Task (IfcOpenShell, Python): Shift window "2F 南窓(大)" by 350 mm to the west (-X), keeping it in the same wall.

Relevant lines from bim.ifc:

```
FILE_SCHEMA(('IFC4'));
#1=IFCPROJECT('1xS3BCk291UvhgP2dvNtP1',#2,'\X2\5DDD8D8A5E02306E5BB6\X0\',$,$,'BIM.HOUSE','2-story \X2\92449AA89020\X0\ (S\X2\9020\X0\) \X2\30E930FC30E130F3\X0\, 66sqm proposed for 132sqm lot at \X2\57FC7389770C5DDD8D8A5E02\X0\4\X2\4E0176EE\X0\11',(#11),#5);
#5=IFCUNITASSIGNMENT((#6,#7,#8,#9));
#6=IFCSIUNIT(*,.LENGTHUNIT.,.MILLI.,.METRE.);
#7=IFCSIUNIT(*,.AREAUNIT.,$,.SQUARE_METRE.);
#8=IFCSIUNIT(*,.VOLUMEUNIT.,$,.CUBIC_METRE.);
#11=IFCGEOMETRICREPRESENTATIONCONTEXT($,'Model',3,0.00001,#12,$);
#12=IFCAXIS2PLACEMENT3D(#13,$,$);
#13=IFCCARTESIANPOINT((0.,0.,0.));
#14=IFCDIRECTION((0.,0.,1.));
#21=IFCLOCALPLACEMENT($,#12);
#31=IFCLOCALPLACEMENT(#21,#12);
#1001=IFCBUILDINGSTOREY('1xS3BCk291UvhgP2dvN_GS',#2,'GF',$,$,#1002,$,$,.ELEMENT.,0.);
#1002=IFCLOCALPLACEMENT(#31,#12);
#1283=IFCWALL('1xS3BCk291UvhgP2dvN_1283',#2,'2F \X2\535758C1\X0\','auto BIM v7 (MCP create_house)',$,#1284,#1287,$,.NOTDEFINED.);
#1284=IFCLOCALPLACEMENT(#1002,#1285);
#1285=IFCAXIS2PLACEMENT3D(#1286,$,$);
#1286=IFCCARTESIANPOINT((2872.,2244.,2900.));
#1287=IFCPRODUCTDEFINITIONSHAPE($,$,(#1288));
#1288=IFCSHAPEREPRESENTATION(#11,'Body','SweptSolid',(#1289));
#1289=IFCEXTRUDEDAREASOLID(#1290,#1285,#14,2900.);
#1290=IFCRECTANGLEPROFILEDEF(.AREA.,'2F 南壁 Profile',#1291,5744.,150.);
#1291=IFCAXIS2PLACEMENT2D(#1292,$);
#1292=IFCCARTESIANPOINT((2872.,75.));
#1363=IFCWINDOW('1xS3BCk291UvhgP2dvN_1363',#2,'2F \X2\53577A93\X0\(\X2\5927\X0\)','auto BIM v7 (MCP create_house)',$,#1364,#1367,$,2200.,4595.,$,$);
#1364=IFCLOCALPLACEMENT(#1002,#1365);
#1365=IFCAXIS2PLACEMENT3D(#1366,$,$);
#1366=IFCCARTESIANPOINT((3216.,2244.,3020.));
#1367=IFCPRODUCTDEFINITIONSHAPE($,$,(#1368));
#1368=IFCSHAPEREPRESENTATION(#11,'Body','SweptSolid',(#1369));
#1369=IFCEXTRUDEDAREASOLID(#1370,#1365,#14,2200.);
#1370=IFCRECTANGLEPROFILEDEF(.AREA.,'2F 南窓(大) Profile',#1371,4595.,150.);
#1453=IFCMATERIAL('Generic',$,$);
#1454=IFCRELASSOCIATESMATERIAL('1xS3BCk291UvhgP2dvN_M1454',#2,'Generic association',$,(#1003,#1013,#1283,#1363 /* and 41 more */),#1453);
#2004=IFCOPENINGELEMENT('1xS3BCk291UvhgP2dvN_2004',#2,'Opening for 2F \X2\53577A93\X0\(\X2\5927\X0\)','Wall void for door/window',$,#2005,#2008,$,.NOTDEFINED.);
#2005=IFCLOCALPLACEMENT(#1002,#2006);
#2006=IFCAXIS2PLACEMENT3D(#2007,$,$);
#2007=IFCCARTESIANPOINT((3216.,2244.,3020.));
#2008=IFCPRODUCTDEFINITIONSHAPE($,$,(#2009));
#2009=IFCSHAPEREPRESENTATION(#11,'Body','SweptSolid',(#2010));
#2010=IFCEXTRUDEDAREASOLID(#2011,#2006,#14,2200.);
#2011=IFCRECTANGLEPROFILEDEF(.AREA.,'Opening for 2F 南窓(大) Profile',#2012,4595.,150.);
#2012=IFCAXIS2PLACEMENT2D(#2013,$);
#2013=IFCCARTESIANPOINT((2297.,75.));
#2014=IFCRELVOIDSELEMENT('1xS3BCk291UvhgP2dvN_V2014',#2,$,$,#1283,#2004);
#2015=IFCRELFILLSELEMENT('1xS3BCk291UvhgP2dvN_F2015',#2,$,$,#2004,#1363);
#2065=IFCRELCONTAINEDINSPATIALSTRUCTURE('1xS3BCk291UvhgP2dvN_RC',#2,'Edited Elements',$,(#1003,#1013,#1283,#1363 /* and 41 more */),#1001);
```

```python
import ifcopenshell
import ifcopenshell.api.geometry
import ifcopenshell.util.placement
import ifcopenshell.util.unit

model = ifcopenshell.open("bim.ifc")
unit_scale = ifcopenshell.util.unit.calculate_unit_scale(model)

window = model.by_id(1363)
opening = window.FillsVoids[0].RelatingOpeningElement
wall = opening.VoidsElements[0].RelatingBuildingElement

wall_matrix = ifcopenshell.util.placement.get_local_placement(wall.ObjectPlacement)
shift = wall_matrix[:3, 0] * -0.35 / unit_scale
before = ifcopenshell.util.placement.get_local_placement(window.ObjectPlacement)[:3, 3].copy()

# The window is not placed relative to its opening, so move both.
for product in (opening, window):
    matrix = ifcopenshell.util.placement.get_local_placement(product.ObjectPlacement)
    matrix[:3, 3] += shift
    ifcopenshell.api.geometry.edit_object_placement(model, product=product, matrix=matrix, is_si=False)

after = ifcopenshell.util.placement.get_local_placement(window.ObjectPlacement)[:3, 3]
print("window moved by", (after - before).round(3) + 0.0)

model.write("bim_v2.ifc")
```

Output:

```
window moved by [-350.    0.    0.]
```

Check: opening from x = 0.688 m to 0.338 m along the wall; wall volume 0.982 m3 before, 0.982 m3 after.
